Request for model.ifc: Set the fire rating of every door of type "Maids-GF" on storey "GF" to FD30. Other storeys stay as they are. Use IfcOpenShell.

First a look at what the model holds.

```python
import ifcopenshell
import ifcopenshell.util.element

model = ifcopenshell.open("model.ifc")
print(model.schema)
storey = next(s for s in model.by_type("IfcBuildingStorey") if s.Name == "GF")
doors = [e for e in ifcopenshell.util.element.get_decomposition(storey) if e.is_a("IfcDoor")]
seen = {}
for e in doors:
    element_type = ifcopenshell.util.element.get_type(e)
    key = (element_type.Name if element_type != e and element_type else None, ifcopenshell.util.element.get_pset(e, "Pset_DoorCommon", "FireRating"))
    seen[key] = seen.get(key, 0) + 1
for (name, value), count in sorted(seen.items(), key=str):
    print(count, "x", name, "|", value)
```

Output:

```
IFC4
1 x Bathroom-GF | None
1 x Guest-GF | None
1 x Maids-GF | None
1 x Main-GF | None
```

```python
import ifcopenshell
import ifcopenshell.api.pset
import ifcopenshell.util.element

model = ifcopenshell.open("model.ifc")

storey = next(s for s in model.by_type("IfcBuildingStorey") if s.Name == "GF")
doors = [e for e in ifcopenshell.util.element.get_decomposition(storey) if e.is_a("IfcDoor")]

count = 0
for e in doors:
    element_type = ifcopenshell.util.element.get_type(e)
    if element_type in (None, e) or element_type.Name != "Maids-GF":
        continue
    # add_pset returns the element's existing set when there is one.
    pset = ifcopenshell.api.pset.add_pset(model, product=e, name="Pset_DoorCommon")
    ifcopenshell.api.pset.edit_pset(model, pset=pset, properties={"FireRating": "FD30"})
    count += 1

print(count, "doors updated")

model.write("model_v2.ifc")
```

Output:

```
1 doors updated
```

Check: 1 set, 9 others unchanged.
